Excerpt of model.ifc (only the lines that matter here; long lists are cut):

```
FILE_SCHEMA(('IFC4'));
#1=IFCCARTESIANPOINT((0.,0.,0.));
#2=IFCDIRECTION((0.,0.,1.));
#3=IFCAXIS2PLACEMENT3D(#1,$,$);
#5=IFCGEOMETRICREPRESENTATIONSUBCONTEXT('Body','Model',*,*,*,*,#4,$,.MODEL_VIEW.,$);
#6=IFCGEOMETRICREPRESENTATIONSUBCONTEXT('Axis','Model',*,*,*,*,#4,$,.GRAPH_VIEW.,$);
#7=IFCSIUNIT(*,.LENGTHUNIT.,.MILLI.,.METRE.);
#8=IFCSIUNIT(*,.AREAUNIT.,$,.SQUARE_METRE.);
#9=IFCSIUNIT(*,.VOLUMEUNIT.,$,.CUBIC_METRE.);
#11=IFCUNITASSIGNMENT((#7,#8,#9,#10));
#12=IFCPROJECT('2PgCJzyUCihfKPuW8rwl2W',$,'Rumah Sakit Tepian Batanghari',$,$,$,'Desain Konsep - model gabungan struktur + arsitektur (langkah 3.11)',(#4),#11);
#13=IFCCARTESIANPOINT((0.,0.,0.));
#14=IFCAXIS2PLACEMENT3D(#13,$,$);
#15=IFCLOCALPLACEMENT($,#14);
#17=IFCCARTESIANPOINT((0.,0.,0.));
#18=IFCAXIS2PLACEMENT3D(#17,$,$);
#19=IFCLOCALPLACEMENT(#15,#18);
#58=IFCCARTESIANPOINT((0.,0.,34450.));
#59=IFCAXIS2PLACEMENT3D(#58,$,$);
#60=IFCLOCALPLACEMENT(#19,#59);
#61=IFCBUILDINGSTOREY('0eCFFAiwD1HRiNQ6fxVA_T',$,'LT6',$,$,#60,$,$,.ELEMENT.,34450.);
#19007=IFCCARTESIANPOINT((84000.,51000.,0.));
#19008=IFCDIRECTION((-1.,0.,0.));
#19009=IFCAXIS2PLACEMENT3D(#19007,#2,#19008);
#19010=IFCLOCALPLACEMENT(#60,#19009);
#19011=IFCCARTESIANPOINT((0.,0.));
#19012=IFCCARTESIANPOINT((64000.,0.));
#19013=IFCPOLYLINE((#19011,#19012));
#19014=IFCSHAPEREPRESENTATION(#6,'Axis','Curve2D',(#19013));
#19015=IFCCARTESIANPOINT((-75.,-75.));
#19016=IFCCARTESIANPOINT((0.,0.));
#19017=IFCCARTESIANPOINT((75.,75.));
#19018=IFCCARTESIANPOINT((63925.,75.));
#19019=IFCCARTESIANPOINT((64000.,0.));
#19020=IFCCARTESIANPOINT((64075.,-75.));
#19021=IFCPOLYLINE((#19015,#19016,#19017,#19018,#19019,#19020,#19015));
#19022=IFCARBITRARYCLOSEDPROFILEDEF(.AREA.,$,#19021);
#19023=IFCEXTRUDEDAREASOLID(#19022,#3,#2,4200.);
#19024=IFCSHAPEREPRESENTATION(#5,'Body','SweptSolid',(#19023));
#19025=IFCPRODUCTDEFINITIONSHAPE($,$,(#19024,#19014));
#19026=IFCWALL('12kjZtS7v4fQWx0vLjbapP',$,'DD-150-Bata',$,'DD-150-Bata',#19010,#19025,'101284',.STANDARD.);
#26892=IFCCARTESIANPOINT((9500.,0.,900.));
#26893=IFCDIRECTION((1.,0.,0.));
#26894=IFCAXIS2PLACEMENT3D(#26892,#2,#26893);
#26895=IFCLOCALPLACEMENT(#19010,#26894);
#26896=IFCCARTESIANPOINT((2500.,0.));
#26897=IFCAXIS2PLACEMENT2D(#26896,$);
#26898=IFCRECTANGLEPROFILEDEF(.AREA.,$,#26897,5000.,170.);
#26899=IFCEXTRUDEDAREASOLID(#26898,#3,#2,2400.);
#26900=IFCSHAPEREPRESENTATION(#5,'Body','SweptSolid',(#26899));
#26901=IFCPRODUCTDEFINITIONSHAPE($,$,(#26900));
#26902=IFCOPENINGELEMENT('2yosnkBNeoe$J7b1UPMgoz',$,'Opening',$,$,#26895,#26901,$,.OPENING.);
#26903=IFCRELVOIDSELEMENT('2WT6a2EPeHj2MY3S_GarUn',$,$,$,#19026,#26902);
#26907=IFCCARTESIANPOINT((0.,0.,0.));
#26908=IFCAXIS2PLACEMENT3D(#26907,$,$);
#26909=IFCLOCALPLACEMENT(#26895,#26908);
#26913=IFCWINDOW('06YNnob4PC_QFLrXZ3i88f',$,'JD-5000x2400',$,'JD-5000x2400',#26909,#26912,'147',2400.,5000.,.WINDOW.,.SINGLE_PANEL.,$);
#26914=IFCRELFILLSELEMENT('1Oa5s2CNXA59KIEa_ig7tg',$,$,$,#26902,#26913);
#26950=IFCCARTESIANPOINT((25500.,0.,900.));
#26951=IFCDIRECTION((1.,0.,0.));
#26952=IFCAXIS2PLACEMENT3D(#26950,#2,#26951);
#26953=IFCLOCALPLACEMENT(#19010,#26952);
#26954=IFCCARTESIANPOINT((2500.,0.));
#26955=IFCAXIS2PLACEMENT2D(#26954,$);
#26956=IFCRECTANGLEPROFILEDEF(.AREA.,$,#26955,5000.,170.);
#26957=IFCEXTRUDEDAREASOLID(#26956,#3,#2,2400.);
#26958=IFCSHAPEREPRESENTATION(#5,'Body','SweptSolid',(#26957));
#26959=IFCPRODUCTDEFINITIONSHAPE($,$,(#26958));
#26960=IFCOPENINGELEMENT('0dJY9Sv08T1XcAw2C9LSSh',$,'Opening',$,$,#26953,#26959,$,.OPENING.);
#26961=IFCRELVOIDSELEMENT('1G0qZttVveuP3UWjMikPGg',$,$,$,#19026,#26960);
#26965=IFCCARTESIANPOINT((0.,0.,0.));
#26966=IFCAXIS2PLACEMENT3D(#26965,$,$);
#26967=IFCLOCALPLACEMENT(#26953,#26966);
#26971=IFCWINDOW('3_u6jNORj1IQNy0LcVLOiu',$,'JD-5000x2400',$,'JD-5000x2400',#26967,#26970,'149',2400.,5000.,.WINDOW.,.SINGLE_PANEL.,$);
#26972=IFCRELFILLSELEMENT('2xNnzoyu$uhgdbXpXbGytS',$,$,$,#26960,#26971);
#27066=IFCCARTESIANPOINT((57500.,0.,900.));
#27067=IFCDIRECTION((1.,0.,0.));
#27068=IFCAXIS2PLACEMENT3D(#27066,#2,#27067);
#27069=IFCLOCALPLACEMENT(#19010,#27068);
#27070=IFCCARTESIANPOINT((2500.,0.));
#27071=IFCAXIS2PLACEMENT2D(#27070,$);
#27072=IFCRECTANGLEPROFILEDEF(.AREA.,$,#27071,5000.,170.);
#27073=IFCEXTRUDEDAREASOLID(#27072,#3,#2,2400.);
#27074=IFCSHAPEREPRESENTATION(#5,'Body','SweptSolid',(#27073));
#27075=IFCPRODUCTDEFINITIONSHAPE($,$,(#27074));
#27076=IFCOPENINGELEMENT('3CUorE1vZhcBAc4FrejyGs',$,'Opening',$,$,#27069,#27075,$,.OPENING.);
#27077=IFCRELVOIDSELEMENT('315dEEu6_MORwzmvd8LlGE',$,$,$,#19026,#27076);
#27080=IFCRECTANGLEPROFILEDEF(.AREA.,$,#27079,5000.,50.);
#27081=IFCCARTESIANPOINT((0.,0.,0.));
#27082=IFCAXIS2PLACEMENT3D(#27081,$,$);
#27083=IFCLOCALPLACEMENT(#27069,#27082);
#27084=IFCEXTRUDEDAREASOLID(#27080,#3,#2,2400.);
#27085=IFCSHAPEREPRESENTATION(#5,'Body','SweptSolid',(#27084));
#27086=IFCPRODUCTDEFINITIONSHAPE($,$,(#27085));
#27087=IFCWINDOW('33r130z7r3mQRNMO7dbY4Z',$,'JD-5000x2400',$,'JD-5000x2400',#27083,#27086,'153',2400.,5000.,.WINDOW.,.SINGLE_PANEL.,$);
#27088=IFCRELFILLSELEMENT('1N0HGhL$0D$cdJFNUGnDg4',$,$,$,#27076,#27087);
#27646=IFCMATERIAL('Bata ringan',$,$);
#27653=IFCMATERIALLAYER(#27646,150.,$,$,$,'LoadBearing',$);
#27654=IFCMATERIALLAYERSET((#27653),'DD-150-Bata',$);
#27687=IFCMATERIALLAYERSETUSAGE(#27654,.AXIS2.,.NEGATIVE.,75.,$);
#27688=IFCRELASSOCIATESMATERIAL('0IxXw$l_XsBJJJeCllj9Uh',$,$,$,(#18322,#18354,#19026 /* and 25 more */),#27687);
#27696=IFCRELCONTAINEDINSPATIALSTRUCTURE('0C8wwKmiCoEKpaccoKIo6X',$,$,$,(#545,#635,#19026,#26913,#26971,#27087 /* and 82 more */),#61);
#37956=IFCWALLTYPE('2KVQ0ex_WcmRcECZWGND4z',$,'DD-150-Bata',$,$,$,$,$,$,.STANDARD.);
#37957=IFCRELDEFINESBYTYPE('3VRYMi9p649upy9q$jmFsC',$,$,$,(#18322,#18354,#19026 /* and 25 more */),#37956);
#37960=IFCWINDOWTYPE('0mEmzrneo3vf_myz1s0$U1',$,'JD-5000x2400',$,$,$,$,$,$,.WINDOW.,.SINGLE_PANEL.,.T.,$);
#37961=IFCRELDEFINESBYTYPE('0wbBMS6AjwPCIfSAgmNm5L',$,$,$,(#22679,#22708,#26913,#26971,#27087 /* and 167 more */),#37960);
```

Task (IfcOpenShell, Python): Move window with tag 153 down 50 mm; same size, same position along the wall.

```python
import numpy as np
import ifcopenshell
import ifcopenshell.api.geometry
import ifcopenshell.util.placement
import ifcopenshell.util.unit

model = ifcopenshell.open("model.ifc")
unit_scale = ifcopenshell.util.unit.calculate_unit_scale(model)

window = model.by_guid("33r130z7r3mQRNMO7dbY4Z")
opening = window.FillsVoids[0].RelatingOpeningElement
dz = -50.0

shift = np.array([0.0, 0.0, dz])
# The window is placed relative to its opening, so it follows when the opening moves.
matrix = ifcopenshell.util.placement.get_local_placement(opening.ObjectPlacement)
matrix[:3, 3] += shift
ifcopenshell.api.geometry.edit_object_placement(
    model, product=opening, matrix=matrix, is_si=False, should_transform_children=True
)

print(f"moved by {dz * unit_scale:+.3f} m")

model.write("model_v2.ifc")
```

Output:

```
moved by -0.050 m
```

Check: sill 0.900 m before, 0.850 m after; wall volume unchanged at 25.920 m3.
